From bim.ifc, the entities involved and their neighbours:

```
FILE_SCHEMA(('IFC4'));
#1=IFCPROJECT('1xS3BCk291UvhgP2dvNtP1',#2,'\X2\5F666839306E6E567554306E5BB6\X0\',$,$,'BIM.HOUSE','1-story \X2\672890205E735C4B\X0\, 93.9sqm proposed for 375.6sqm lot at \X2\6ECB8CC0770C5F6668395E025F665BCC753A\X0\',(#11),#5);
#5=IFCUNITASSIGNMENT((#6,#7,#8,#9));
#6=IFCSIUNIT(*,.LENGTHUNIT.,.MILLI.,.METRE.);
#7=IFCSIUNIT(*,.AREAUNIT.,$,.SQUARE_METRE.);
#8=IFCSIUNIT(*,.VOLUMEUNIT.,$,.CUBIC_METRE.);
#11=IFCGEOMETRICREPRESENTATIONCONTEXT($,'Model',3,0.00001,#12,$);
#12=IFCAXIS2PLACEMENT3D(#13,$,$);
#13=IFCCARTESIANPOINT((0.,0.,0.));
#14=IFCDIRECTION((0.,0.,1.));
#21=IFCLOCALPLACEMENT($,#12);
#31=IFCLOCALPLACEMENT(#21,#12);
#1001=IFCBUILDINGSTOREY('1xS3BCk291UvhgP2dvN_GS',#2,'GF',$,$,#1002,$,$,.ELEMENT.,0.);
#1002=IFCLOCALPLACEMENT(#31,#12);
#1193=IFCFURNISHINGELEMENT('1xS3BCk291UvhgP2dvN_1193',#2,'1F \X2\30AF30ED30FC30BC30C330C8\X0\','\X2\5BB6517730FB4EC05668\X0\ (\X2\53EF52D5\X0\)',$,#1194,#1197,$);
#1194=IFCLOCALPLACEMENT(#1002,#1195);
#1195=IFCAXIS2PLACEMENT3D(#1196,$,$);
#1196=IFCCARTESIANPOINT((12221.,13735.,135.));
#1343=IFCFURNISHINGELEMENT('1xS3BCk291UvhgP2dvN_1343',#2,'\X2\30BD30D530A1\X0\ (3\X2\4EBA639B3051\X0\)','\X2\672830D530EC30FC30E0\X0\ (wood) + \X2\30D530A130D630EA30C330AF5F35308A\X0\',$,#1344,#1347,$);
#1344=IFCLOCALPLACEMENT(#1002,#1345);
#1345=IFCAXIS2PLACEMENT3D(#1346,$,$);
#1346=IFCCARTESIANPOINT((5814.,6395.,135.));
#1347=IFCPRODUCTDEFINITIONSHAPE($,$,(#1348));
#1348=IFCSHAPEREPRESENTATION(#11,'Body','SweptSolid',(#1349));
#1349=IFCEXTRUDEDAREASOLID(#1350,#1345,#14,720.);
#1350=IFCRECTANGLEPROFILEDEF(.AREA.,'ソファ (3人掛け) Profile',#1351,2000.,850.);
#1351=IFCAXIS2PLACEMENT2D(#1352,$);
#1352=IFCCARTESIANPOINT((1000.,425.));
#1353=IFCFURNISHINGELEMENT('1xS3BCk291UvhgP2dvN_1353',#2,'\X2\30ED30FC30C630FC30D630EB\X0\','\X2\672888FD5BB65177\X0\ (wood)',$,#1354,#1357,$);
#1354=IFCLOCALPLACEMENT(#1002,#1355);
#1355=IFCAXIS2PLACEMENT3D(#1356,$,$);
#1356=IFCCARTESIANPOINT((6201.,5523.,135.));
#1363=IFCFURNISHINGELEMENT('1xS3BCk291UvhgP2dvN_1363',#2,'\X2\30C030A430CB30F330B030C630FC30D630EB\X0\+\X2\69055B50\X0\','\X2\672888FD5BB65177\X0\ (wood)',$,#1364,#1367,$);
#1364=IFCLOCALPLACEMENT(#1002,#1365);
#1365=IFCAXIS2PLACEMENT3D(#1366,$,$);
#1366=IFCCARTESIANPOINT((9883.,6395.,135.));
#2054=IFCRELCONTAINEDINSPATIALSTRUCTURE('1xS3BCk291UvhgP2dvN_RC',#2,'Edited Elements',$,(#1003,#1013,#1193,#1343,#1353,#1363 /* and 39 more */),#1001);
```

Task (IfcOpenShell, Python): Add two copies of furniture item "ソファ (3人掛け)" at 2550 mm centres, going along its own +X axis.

```python
import ifcopenshell
import ifcopenshell.api.geometry
import ifcopenshell.api.root
import ifcopenshell.util.element
import ifcopenshell.util.placement

model = ifcopenshell.open("bim.ifc")


def reuse_history(source, copy):
    """copy_class also copies each property set's owner history, people and application; keep the originals."""
    for rel in copy.IsDefinedBy:
        if rel.is_a("IfcRelDefinesByProperties") and (history := rel.RelatingPropertyDefinition.OwnerHistory):
            rel.RelatingPropertyDefinition.OwnerHistory = source.OwnerHistory
            ifcopenshell.util.element.remove_deep2(model, history)


source = model.by_id(1343)
base = ifcopenshell.util.placement.get_local_placement(source.ObjectPlacement)
step = base[:3, 0] * 2550.0

for i in range(1, 3):
    copy = ifcopenshell.api.root.copy_class(model, product=source)
    copy.Representation = ifcopenshell.util.element.copy_deep(
        model, source.Representation, exclude=["IfcGeometricRepresentationContext", "IfcRepresentationMap"]
    )
    reuse_history(source, copy)
    matrix = base.copy()
    matrix[:3, 3] += i * step
    print("added at", matrix[:3, 3].round(3) + 0.0)
    ifcopenshell.api.geometry.edit_object_placement(model, product=copy, matrix=matrix, is_si=False)

model.write("bim_edited.ifc")
```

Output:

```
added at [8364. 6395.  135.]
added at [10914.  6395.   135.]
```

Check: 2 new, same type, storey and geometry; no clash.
